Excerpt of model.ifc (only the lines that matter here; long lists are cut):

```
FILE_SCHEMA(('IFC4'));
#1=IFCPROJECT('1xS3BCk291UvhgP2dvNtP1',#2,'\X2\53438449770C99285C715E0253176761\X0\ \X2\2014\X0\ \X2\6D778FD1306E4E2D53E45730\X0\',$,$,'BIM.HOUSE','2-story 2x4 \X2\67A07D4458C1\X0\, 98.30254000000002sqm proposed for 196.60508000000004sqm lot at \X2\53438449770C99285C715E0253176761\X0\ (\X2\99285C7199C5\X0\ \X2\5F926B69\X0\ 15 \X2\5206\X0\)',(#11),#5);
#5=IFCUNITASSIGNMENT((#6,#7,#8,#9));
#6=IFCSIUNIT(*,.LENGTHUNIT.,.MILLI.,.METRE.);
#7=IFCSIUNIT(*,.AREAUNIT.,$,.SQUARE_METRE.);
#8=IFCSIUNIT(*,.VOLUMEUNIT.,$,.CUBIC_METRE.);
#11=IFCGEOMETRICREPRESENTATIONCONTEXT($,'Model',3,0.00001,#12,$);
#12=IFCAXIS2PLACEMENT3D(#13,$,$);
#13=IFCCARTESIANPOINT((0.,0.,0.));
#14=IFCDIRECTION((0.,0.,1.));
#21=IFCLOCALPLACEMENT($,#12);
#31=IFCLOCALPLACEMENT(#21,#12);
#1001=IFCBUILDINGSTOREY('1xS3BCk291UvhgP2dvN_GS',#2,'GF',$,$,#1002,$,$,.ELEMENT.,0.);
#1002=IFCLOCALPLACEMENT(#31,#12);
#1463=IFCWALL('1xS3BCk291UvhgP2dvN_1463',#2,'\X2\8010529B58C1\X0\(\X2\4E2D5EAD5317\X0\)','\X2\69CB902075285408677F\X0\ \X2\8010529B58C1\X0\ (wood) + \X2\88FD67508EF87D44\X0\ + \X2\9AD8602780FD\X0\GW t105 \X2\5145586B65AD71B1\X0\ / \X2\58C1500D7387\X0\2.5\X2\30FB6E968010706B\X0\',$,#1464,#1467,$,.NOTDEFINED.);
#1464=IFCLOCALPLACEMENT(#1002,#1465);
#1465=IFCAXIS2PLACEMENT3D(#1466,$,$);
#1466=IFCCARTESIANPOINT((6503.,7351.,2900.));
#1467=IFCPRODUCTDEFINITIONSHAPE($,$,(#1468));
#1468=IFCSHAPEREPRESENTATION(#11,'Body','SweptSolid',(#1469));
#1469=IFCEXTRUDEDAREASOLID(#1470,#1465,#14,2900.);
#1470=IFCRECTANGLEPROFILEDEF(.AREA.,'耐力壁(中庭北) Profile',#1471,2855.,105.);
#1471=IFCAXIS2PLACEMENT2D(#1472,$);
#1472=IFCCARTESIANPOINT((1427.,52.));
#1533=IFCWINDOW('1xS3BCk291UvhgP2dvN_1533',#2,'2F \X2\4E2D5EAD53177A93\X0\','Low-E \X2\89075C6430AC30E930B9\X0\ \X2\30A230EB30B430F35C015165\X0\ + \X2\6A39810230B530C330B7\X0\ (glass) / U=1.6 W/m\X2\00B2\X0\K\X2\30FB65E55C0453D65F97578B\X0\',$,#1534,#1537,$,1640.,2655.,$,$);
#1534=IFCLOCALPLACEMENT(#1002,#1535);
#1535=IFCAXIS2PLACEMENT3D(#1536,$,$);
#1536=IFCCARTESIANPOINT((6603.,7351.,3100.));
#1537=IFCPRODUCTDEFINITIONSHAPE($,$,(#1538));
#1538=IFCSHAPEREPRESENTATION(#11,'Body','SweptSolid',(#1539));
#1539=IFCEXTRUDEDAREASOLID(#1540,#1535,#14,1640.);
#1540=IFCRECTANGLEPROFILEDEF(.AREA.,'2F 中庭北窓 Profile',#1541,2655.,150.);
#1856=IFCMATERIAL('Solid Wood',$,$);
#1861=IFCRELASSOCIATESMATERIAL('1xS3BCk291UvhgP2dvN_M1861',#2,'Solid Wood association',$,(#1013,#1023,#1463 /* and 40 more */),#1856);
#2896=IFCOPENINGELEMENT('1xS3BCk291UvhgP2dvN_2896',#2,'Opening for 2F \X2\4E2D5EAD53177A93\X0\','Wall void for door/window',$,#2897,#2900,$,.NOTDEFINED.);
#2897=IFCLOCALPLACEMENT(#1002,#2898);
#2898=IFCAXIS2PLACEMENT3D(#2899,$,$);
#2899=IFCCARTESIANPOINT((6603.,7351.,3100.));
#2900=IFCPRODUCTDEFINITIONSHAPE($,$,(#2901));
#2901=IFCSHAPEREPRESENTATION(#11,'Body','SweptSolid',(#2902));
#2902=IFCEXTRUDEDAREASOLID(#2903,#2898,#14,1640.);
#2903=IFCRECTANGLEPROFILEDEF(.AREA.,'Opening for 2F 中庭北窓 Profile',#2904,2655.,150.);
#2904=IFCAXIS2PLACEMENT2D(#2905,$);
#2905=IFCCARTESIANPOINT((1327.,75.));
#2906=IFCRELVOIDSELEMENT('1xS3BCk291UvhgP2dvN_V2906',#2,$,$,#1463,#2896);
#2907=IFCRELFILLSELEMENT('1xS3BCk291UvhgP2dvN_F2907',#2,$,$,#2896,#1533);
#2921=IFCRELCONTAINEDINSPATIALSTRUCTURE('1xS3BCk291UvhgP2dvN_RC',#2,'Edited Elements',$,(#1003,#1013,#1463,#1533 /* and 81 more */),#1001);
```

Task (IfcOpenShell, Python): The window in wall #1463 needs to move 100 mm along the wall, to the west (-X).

```python
import ifcopenshell
import ifcopenshell.api.geometry
import ifcopenshell.util.placement
import ifcopenshell.util.unit

model = ifcopenshell.open("model.ifc")
unit_scale = ifcopenshell.util.unit.calculate_unit_scale(model)

window = model.by_guid("1xS3BCk291UvhgP2dvN_1533")
opening = window.FillsVoids[0].RelatingOpeningElement
wall = opening.VoidsElements[0].RelatingBuildingElement

wall_matrix = ifcopenshell.util.placement.get_local_placement(wall.ObjectPlacement)
shift = wall_matrix[:3, 0] * -0.1 / unit_scale
before = ifcopenshell.util.placement.get_local_placement(window.ObjectPlacement)[:3, 3].copy()

# The window is not placed relative to its opening, so move both.
for product in (opening, window):
    matrix = ifcopenshell.util.placement.get_local_placement(product.ObjectPlacement)
    matrix[:3, 3] += shift
    ifcopenshell.api.geometry.edit_object_placement(model, product=product, matrix=matrix, is_si=False)

after = ifcopenshell.util.placement.get_local_placement(window.ObjectPlacement)[:3, 3]
print("window moved by", (after - before).round(3) + 0.0)

model.write("model-out.ifc")
```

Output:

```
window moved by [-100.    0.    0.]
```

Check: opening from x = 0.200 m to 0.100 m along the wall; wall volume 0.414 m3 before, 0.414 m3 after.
